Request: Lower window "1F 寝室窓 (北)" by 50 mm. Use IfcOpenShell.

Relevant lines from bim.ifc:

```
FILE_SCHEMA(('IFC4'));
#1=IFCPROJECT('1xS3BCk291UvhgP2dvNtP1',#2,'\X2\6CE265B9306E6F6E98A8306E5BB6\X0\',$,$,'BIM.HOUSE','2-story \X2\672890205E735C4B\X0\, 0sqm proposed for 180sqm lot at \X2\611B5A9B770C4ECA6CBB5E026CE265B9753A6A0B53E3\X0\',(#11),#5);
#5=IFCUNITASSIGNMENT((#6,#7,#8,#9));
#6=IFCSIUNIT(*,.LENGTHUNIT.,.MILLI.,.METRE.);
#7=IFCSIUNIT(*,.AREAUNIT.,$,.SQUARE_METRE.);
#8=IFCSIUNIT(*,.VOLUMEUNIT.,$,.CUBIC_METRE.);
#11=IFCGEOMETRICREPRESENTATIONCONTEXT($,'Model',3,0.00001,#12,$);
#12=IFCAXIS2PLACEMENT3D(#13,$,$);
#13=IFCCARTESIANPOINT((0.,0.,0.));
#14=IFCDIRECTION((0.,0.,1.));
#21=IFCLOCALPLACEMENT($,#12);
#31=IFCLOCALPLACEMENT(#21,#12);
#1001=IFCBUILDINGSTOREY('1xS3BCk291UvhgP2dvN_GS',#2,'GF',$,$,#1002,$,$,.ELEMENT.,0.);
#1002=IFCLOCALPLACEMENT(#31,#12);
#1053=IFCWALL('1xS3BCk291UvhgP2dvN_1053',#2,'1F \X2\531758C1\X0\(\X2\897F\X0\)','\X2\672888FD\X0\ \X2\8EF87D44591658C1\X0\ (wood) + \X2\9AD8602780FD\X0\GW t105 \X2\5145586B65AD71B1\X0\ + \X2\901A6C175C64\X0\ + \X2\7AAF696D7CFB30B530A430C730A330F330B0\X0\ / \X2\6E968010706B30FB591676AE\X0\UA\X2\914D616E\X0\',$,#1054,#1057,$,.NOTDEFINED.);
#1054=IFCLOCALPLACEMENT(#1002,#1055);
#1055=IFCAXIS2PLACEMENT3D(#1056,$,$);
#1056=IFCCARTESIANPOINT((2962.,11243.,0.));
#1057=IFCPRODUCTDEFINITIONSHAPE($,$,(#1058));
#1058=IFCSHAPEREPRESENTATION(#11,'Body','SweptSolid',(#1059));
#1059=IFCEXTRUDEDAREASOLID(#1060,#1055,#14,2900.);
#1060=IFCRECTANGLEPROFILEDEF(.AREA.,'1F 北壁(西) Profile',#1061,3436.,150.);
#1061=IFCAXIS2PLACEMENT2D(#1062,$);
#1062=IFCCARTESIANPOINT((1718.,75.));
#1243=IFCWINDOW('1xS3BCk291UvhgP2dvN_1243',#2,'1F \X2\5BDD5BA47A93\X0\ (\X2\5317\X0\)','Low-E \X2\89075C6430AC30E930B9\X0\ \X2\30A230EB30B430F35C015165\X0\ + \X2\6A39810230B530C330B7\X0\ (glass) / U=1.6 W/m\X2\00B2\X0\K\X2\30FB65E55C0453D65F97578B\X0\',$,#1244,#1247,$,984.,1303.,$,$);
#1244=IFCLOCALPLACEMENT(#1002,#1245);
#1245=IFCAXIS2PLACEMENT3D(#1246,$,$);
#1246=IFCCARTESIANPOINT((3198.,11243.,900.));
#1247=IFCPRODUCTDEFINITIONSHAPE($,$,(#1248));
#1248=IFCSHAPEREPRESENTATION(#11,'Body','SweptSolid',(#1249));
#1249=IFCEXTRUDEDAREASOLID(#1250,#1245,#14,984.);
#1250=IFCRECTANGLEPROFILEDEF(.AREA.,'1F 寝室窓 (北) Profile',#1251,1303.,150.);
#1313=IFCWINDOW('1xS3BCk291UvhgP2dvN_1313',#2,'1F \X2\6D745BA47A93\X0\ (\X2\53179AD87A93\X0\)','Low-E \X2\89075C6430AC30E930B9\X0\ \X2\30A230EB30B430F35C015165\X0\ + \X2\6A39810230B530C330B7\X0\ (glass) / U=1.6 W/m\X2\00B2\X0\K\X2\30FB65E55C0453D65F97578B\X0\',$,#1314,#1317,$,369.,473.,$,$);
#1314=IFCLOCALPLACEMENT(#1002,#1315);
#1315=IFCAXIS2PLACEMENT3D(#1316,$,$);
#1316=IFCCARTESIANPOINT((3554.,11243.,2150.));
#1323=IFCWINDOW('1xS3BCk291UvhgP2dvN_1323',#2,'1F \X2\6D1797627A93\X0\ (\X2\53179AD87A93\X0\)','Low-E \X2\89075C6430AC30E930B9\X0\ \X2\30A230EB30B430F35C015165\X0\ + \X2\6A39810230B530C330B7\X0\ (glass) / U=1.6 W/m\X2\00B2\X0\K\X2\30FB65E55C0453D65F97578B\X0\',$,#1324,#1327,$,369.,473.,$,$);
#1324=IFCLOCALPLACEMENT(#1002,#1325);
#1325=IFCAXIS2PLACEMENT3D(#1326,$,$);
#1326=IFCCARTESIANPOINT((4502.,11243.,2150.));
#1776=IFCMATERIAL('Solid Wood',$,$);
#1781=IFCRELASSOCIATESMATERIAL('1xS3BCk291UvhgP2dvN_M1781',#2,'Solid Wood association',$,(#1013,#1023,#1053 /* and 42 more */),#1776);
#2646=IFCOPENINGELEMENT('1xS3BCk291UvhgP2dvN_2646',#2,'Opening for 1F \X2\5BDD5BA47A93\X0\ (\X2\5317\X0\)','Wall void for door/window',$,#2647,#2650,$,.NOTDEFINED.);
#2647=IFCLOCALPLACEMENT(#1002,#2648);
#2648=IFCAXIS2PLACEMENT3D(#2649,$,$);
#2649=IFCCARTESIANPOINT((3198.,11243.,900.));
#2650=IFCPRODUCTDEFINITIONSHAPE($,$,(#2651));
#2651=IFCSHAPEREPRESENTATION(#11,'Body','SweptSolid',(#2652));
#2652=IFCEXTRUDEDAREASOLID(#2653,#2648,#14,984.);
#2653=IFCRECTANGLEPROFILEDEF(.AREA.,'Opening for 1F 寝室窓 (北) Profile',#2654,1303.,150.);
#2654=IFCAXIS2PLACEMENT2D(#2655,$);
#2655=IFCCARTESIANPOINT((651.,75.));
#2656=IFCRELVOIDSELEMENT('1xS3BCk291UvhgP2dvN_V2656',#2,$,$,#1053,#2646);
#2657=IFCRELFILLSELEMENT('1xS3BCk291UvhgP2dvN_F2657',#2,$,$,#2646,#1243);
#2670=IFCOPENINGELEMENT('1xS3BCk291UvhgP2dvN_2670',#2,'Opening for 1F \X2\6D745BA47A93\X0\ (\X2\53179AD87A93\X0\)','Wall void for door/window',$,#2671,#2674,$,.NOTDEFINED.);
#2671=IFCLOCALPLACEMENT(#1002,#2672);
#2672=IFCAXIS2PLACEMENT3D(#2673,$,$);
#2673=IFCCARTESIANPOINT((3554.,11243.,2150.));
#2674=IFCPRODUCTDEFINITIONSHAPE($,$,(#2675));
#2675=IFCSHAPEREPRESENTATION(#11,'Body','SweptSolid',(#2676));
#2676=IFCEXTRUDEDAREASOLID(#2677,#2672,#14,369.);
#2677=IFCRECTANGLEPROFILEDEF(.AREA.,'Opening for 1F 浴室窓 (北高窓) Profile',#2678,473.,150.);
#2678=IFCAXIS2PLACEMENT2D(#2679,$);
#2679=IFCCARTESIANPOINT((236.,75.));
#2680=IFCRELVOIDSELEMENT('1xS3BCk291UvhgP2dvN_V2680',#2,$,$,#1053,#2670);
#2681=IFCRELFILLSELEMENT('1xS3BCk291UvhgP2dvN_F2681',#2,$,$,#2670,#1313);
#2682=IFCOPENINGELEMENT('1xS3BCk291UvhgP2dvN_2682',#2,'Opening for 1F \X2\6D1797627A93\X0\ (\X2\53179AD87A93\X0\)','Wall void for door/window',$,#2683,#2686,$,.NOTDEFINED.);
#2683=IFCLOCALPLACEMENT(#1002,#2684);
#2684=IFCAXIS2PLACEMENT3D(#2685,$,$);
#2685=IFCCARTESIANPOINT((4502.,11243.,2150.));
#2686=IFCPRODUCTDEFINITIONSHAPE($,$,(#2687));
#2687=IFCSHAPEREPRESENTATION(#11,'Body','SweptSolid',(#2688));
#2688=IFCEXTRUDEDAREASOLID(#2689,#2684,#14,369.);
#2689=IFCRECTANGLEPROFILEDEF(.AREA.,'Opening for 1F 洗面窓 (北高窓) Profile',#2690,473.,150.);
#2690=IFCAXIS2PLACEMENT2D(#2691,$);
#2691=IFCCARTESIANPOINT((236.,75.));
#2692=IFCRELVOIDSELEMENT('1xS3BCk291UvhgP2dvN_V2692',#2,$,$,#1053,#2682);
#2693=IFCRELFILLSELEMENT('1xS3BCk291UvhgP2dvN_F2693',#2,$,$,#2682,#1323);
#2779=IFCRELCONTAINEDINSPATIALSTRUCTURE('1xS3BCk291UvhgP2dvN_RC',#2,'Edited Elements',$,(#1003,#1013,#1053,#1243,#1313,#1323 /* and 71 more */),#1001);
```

```python
import numpy as np
import ifcopenshell
import ifcopenshell.api.geometry
import ifcopenshell.util.placement
import ifcopenshell.util.unit

model = ifcopenshell.open("bim.ifc")
unit_scale = ifcopenshell.util.unit.calculate_unit_scale(model)

window = model.by_id(1243)
opening = window.FillsVoids[0].RelatingOpeningElement
dz = -0.05 / unit_scale

shift = np.array([0.0, 0.0, dz])
# The window is not placed relative to its opening, so move both.
for product in (opening, window):
    matrix = ifcopenshell.util.placement.get_local_placement(product.ObjectPlacement)
    matrix[:3, 3] += shift
    ifcopenshell.api.geometry.edit_object_placement(model, product=product, matrix=matrix, is_si=False)

print(f"moved by {dz * unit_scale:+.3f} m")

model.write("bim_edited.ifc")
```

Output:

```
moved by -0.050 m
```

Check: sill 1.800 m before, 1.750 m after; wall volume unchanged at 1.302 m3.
